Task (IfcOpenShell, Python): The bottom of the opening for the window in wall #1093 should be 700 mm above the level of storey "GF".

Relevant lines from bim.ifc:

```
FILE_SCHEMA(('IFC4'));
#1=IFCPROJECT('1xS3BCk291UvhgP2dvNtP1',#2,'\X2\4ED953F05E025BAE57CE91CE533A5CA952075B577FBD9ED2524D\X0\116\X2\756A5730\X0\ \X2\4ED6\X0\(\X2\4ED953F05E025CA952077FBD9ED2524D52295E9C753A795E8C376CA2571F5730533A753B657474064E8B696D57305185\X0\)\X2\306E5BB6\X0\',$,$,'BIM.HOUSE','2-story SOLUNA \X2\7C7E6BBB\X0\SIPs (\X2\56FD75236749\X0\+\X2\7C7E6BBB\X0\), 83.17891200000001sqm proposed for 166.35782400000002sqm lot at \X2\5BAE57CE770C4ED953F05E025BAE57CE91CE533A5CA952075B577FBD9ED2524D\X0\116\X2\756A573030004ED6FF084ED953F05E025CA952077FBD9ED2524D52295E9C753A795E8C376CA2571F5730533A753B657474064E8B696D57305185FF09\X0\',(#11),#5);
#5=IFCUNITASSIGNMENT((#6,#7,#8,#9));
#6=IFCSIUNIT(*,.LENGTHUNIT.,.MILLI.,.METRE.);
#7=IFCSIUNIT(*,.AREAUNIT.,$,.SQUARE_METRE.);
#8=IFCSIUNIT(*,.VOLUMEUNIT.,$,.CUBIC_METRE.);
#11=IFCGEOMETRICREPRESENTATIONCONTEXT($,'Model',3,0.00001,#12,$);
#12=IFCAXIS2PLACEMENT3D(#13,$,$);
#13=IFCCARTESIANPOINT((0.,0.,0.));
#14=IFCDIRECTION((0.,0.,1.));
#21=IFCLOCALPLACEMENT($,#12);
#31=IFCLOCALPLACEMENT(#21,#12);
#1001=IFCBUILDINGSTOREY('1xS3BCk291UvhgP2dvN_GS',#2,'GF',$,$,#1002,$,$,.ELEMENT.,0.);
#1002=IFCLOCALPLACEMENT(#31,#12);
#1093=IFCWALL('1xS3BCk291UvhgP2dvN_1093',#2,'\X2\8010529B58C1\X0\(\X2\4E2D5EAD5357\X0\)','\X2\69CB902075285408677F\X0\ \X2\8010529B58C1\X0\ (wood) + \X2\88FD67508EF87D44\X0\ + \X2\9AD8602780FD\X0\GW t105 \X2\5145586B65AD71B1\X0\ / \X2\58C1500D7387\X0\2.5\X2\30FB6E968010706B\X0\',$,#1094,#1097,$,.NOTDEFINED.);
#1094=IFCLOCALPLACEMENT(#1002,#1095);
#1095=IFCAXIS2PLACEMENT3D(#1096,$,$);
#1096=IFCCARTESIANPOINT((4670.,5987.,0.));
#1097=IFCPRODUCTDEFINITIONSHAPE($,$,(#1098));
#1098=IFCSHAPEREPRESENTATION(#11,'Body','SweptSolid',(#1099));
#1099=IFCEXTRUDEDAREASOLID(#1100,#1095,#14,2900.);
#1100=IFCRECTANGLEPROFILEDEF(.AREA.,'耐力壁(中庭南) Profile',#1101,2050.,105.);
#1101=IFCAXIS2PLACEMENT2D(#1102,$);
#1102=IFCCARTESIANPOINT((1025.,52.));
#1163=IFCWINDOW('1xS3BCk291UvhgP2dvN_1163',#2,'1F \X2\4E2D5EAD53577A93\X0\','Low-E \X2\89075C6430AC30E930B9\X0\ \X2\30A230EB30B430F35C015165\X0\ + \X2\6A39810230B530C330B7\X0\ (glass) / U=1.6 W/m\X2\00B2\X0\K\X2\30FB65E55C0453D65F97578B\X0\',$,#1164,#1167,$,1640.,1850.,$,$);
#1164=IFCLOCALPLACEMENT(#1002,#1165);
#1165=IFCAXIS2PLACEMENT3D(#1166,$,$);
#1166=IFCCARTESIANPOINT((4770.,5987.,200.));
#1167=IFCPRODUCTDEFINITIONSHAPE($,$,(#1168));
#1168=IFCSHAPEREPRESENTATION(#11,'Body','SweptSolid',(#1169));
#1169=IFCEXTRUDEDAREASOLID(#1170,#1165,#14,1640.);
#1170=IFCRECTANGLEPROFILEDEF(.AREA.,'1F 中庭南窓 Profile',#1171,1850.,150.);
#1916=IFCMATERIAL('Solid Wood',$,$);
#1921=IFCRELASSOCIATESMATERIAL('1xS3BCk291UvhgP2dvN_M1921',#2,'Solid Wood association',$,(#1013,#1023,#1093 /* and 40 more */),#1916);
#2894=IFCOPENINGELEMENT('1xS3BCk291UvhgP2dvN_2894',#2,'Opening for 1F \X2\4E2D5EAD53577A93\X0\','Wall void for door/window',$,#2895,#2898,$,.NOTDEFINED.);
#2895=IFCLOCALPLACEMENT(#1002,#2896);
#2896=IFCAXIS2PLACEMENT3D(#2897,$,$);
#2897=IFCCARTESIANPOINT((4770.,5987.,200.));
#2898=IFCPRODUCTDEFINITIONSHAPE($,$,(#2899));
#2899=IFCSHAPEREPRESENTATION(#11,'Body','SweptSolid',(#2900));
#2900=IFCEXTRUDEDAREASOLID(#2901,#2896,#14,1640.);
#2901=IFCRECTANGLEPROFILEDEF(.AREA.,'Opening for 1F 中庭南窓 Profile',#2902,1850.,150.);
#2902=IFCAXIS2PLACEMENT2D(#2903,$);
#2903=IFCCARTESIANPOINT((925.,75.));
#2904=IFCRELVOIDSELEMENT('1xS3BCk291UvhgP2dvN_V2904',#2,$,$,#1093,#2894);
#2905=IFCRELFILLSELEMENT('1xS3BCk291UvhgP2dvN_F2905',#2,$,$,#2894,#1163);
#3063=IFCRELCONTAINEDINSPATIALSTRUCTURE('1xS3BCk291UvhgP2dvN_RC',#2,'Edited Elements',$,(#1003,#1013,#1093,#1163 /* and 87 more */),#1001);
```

```python
import numpy as np
import ifcopenshell
import ifcopenshell.api.geometry
import ifcopenshell.geom
import ifcopenshell.util.element
import ifcopenshell.util.placement
import ifcopenshell.util.shape
import ifcopenshell.util.unit

model = ifcopenshell.open("bim.ifc")
unit_scale = ifcopenshell.util.unit.calculate_unit_scale(model)

window = model.by_guid("1xS3BCk291UvhgP2dvN_1163")
opening = window.FillsVoids[0].RelatingOpeningElement
storey = ifcopenshell.util.element.get_container(window, ifc_class="IfcBuildingStorey")
level = ifcopenshell.util.placement.get_local_placement(storey.ObjectPlacement)[2, 3]

# The opening's origin need not be at the sill, so measure its lowest point.
shape = ifcopenshell.geom.create_shape(ifcopenshell.geom.settings(), opening)
bottom = ifcopenshell.util.shape.get_shape_bottom_elevation(shape, shape.geometry) / unit_scale
dz = level + 0.7 / unit_scale - bottom

shift = np.array([0.0, 0.0, dz])
# The window is not placed relative to its opening, so move both.
for product in (opening, window):
    matrix = ifcopenshell.util.placement.get_local_placement(product.ObjectPlacement)
    matrix[:3, 3] += shift
    ifcopenshell.api.geometry.edit_object_placement(model, product=product, matrix=matrix, is_si=False)

print(f"moved by {dz * unit_scale:+.3f} m")

model.write("bim_updated.ifc")
```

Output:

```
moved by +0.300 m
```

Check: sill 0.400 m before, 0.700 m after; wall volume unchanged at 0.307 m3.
